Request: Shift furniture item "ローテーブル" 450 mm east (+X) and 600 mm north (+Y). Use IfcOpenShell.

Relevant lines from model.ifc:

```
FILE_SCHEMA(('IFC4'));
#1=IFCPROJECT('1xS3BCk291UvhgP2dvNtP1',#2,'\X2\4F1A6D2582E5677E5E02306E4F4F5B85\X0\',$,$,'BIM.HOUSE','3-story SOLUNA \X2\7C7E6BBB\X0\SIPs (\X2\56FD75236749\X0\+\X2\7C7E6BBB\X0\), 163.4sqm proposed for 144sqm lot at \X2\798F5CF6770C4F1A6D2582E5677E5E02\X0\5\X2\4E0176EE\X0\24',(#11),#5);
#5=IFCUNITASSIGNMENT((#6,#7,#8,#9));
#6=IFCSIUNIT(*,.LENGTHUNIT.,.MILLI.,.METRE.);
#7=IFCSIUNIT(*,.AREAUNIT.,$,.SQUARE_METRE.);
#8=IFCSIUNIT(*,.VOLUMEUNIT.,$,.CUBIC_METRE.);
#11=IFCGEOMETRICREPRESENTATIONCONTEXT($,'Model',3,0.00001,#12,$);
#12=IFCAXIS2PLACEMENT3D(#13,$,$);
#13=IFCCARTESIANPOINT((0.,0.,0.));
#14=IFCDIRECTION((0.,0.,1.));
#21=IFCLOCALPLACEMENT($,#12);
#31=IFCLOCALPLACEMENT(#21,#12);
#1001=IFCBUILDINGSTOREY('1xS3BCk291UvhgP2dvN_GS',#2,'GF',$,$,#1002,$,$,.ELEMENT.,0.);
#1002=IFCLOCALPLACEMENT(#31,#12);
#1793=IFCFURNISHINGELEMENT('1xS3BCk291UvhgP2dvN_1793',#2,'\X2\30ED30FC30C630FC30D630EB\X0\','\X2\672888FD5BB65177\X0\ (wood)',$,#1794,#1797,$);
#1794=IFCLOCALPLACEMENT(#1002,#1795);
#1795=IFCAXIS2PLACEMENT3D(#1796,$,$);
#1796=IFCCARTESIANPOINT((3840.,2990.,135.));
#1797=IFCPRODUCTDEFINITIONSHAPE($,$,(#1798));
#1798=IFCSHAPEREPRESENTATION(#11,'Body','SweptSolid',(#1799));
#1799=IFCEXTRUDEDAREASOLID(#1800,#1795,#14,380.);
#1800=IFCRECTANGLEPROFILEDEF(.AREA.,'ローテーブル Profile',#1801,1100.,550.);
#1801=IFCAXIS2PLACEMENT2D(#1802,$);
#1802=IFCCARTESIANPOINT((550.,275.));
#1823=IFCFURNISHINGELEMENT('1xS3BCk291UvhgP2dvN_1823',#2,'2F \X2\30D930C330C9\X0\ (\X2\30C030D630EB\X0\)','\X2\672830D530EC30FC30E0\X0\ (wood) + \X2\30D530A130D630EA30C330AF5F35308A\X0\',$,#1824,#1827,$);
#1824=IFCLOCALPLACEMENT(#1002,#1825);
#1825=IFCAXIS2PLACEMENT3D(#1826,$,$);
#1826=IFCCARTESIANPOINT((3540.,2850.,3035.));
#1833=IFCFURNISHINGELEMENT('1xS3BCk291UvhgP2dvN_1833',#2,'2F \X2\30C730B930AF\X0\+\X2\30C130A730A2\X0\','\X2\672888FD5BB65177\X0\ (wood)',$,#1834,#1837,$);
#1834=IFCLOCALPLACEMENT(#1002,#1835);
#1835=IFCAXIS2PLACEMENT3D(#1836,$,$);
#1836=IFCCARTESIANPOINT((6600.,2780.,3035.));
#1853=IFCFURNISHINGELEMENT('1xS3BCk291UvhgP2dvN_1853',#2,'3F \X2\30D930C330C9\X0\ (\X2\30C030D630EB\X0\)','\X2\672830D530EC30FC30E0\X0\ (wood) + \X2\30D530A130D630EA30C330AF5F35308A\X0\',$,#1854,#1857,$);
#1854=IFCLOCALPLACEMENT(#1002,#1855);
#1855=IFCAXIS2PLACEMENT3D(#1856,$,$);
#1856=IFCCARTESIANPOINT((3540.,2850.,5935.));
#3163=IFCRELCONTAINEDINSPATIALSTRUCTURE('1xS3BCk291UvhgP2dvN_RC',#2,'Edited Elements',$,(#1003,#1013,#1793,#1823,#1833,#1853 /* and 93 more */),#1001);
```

```python
import ifcopenshell
import ifcopenshell.api.geometry
import ifcopenshell.util.placement
import ifcopenshell.util.unit

model = ifcopenshell.open("model.ifc")
unit_scale = ifcopenshell.util.unit.calculate_unit_scale(model)

item = model.by_guid("1xS3BCk291UvhgP2dvN_1793")
matrix = ifcopenshell.util.placement.get_local_placement(item.ObjectPlacement)
matrix[0, 3] += 0.45 / unit_scale
matrix[1, 3] += 0.6 / unit_scale
ifcopenshell.api.geometry.edit_object_placement(model, product=item, matrix=matrix, is_si=False)

print(ifcopenshell.util.placement.get_local_placement(item.ObjectPlacement).round(3) + 0.0)

model.write("model_edited.ifc")
```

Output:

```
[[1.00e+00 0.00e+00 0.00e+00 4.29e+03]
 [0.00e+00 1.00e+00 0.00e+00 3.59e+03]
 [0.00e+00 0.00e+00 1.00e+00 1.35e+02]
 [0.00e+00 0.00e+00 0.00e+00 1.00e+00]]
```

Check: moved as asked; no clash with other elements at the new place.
